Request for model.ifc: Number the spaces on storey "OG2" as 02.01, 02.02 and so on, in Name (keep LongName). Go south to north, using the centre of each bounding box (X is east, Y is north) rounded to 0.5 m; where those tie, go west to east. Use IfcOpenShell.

First a look at what the model holds.

```python
import ifcopenshell
import ifcopenshell.util.element
import ifcopenshell.util.placement

model = ifcopenshell.open("model.ifc")
print(model.schema)
storey = next(s for s in model.by_type("IfcBuildingStorey") if s.Name == "OG2")
spaces = [e for e in ifcopenshell.util.element.get_decomposition(storey) if e.is_a("IfcSpace")]
for e in sorted(spaces, key=lambda e: e.id()):
    origin = ifcopenshell.util.placement.get_local_placement(e.ObjectPlacement)[:3, 3]
    print(e.id(), e.Name, e.LongName, origin.round(2) + 0.0, sep=" | ")
```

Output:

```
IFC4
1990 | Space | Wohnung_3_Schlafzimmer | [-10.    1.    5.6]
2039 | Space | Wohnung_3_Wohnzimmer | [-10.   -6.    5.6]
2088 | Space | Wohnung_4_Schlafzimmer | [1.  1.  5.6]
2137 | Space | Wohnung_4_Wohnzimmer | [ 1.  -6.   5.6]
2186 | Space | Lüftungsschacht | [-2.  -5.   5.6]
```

```python
import ifcopenshell
import ifcopenshell.geom
import ifcopenshell.util.element
import ifcopenshell.util.shape

model = ifcopenshell.open("model.ifc")
settings = ifcopenshell.geom.settings()
settings.set("use-world-coords", True)


def centre(element):
    shape = ifcopenshell.geom.create_shape(settings, element)
    return ifcopenshell.util.shape.get_bbox_centroid(shape.geometry)


storey = next(s for s in model.by_type("IfcBuildingStorey") if s.Name == "OG2")
spaces = [e for e in ifcopenshell.util.element.get_decomposition(storey) if e.is_a("IfcSpace")]

# Insertion points can sit at a corner or the storey origin, so sort by the geometry (in metres).
centres = {e: centre(e) for e in spaces}
spaces.sort(key=lambda e: (round(centres[e][1] / 0.5), centres[e][0]))

for i, e in enumerate(spaces, start=1):
    number = f"02.{i:02d}"
    e.Name = number
    print(e.id(), number)

model.write("model_updated.ifc")
```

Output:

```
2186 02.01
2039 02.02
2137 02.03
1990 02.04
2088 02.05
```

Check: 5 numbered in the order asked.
